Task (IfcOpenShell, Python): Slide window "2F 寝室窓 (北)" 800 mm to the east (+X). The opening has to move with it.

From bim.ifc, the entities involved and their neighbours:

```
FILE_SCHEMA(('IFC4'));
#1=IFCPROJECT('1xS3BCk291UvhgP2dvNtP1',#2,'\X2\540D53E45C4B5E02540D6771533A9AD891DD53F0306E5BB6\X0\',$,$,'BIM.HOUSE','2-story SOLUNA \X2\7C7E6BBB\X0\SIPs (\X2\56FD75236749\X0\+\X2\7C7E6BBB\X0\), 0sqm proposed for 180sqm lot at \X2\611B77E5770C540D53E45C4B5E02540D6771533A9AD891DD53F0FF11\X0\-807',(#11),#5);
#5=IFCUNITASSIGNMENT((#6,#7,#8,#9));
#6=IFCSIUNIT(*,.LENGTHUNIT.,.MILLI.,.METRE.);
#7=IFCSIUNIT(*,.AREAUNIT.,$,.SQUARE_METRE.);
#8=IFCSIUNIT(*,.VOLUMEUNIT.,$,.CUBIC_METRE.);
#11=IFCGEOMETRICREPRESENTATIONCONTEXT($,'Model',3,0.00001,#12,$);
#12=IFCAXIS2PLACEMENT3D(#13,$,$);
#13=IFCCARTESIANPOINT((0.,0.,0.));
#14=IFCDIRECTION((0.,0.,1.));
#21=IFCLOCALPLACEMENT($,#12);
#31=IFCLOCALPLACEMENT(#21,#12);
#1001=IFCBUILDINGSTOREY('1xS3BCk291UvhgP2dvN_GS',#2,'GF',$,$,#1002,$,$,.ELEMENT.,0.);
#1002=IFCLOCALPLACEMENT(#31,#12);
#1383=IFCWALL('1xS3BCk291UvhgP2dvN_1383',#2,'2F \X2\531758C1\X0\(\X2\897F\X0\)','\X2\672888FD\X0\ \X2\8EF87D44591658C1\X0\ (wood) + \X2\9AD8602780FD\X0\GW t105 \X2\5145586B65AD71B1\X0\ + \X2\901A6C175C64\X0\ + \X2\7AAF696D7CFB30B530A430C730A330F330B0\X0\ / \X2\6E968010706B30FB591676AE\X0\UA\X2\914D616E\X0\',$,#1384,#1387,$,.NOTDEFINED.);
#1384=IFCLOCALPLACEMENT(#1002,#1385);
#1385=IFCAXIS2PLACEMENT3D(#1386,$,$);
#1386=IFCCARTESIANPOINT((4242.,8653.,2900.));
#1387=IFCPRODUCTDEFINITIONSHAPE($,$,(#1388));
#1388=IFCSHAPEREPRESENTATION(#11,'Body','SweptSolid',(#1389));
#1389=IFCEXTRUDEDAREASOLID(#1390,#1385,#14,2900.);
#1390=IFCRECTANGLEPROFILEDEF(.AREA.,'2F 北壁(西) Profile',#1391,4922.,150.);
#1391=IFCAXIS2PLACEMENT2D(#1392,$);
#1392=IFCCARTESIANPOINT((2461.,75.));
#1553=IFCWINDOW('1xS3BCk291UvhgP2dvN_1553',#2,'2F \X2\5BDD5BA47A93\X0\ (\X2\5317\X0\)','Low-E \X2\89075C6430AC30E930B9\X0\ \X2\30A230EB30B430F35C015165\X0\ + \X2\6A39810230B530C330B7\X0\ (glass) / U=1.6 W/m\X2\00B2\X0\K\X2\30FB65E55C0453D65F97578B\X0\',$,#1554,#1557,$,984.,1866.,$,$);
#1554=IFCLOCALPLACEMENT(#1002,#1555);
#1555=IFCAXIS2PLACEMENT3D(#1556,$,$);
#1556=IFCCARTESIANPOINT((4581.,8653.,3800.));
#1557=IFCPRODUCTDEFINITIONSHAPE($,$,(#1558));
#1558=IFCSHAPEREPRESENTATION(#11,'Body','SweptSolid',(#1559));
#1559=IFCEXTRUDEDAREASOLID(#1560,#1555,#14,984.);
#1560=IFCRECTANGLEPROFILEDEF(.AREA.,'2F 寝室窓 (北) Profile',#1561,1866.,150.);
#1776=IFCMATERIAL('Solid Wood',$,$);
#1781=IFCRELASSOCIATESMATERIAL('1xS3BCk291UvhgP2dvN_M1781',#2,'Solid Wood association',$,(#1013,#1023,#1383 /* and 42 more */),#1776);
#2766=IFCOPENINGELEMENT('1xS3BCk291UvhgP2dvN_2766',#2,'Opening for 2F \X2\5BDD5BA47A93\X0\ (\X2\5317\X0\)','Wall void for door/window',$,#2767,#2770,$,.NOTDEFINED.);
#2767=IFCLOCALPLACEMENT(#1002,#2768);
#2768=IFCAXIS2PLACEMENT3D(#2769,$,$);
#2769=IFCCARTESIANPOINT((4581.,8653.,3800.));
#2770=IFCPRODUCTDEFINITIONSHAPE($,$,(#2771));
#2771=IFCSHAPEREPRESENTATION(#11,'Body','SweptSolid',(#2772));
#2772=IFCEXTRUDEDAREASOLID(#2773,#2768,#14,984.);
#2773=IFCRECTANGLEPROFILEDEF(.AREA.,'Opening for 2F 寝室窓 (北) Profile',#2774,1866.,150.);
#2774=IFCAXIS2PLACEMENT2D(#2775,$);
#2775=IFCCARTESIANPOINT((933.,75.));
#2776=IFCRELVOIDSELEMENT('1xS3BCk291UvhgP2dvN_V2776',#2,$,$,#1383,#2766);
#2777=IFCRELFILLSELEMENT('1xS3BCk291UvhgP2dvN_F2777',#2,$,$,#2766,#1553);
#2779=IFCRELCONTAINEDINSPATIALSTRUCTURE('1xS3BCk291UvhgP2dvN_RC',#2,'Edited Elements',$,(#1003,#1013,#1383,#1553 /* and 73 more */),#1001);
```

```python
import ifcopenshell
import ifcopenshell.api.geometry
import ifcopenshell.util.placement

model = ifcopenshell.open("bim.ifc")

window = model.by_guid("1xS3BCk291UvhgP2dvN_1553")
opening = window.FillsVoids[0].RelatingOpeningElement
wall = opening.VoidsElements[0].RelatingBuildingElement

wall_matrix = ifcopenshell.util.placement.get_local_placement(wall.ObjectPlacement)
shift = wall_matrix[:3, 0] * 800.0
before = ifcopenshell.util.placement.get_local_placement(window.ObjectPlacement)[:3, 3].copy()

# The window is not placed relative to its opening, so move both.
for product in (opening, window):
    matrix = ifcopenshell.util.placement.get_local_placement(product.ObjectPlacement)
    matrix[:3, 3] += shift
    ifcopenshell.api.geometry.edit_object_placement(model, product=product, matrix=matrix, is_si=False)

after = ifcopenshell.util.placement.get_local_placement(window.ObjectPlacement)[:3, 3]
print("window moved by", (after - before).round(3) + 0.0)

model.write("bim_edited.ifc")
```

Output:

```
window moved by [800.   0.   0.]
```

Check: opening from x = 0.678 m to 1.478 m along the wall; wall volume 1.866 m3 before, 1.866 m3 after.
